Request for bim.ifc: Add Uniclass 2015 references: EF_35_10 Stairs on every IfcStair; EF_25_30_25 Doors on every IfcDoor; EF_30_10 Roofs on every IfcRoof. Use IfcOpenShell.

First a look at what the model holds.

```python
import ifcopenshell

model = ifcopenshell.open("bim.ifc")
print(model.schema)
print("classifications:", [c.Name for c in model.by_type("IfcClassification")])
for ifc_class in ("IfcDoor", "IfcRoof", "IfcStair", "IfcWall", "IfcWindow"):
    print(ifc_class, len(model.by_type(ifc_class)))
```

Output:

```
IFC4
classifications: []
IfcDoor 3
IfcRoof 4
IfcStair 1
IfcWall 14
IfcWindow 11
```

```python
import ifcopenshell
import ifcopenshell.api.classification

model = ifcopenshell.open("bim.ifc")

system = ifcopenshell.api.classification.add_classification(model, classification="Uniclass 2015")

codes = {
    "IfcStair": ("EF_35_10", "Stairs"),
    "IfcDoor": ("EF_25_30_25", "Doors"),
    "IfcRoof": ("EF_30_10", "Roofs"),
}
for ifc_class, (code, name) in codes.items():
    products = model.by_type(ifc_class)
    ifcopenshell.api.classification.add_reference(
        model, products=products, classification=system, identification=code, name=name
    )
    print(code, len(products))

model.write("bim-out.ifc")
```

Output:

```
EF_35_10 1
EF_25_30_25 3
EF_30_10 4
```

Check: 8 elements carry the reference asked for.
